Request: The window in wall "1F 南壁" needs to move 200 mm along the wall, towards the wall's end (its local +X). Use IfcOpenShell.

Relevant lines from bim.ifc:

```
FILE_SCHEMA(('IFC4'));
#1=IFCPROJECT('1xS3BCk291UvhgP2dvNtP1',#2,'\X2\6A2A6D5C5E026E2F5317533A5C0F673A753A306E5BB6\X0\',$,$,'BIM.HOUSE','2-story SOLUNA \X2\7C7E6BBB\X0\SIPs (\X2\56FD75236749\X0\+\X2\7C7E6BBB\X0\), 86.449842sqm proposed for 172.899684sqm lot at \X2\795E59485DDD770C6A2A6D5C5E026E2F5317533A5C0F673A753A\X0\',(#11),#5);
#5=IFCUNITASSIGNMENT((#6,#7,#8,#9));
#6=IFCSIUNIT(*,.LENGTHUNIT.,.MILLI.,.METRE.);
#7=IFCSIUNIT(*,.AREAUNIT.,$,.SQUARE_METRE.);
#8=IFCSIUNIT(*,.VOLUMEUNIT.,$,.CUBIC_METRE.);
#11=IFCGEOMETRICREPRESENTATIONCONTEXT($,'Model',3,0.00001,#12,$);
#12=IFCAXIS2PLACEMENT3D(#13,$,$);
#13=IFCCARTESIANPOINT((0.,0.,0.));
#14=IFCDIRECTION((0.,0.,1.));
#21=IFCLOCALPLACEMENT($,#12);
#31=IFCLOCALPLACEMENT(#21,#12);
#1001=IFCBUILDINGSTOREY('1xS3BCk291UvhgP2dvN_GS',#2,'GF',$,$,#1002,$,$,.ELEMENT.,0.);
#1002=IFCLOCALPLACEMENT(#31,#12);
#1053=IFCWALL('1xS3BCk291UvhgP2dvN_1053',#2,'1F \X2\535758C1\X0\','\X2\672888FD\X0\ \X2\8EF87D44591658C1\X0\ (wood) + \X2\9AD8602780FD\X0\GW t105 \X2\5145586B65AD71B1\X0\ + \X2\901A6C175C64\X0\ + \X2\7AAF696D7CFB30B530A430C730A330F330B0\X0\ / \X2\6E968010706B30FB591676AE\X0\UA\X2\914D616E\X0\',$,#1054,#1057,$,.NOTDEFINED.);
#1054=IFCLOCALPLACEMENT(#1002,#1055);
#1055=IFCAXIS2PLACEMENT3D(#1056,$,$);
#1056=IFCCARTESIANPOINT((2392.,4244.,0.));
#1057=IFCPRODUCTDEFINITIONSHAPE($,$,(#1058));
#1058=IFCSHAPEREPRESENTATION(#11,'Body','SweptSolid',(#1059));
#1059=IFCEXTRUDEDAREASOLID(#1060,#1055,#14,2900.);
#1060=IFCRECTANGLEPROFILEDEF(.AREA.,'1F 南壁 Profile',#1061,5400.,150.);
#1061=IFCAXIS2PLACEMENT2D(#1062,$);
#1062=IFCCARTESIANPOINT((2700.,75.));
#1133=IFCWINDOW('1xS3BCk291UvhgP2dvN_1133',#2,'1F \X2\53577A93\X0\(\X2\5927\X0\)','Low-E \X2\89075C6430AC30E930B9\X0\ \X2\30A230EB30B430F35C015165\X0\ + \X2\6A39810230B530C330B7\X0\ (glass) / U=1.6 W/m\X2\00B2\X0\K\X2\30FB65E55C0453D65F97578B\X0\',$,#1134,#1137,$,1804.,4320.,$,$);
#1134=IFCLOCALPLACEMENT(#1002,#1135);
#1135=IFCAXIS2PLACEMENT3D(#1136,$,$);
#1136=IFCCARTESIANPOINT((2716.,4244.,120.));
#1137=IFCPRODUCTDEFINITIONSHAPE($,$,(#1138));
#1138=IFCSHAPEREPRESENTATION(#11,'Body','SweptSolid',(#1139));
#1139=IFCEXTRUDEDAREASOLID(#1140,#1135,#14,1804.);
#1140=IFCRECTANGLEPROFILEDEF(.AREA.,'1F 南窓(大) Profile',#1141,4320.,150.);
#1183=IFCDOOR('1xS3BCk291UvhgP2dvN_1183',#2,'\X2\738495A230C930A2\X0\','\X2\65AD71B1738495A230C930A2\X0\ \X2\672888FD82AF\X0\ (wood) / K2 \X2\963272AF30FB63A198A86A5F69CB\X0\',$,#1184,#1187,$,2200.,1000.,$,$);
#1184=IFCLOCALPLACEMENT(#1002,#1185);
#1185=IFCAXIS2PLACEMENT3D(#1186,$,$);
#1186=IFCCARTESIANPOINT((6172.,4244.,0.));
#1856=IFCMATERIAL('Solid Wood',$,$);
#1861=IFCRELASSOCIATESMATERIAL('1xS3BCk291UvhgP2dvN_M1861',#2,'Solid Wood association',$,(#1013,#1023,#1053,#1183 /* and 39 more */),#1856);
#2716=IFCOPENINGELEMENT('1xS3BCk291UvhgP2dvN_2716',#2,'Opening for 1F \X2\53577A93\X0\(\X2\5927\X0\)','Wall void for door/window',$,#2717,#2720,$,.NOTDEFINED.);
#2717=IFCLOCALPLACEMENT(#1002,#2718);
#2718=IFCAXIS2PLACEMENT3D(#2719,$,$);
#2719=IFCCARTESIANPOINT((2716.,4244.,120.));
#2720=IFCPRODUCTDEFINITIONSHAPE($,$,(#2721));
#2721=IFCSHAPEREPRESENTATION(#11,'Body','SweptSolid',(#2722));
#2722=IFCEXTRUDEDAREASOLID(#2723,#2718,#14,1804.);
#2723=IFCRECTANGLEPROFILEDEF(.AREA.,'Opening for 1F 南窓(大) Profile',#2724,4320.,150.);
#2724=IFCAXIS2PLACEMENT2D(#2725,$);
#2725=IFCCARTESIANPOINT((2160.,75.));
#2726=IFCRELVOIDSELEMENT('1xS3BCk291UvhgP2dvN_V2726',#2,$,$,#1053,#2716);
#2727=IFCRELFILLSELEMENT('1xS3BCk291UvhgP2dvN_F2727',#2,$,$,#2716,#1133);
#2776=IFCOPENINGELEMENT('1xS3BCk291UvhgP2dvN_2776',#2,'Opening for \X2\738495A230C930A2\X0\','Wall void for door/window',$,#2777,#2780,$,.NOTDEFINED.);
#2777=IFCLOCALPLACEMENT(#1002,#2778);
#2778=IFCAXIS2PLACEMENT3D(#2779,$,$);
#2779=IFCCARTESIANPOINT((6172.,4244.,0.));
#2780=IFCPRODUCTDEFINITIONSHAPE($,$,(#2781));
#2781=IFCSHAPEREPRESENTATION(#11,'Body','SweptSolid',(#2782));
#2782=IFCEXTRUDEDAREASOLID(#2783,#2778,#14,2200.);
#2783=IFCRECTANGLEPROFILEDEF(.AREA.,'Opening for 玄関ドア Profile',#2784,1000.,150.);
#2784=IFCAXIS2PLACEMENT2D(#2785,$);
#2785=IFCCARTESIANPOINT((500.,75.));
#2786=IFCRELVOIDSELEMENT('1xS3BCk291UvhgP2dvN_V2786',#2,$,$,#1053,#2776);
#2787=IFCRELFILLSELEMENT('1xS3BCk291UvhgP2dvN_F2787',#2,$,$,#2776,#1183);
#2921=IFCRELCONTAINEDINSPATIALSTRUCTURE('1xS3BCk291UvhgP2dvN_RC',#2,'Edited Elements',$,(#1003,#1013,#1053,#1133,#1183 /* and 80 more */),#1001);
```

```python
import ifcopenshell
import ifcopenshell.api.geometry
import ifcopenshell.util.placement
import ifcopenshell.util.unit

model = ifcopenshell.open("bim.ifc")
unit_scale = ifcopenshell.util.unit.calculate_unit_scale(model)

window = model.by_guid("1xS3BCk291UvhgP2dvN_1133")
opening = window.FillsVoids[0].RelatingOpeningElement
wall = opening.VoidsElements[0].RelatingBuildingElement

wall_matrix = ifcopenshell.util.placement.get_local_placement(wall.ObjectPlacement)
shift = wall_matrix[:3, 0] * 0.2 / unit_scale
before = ifcopenshell.util.placement.get_local_placement(window.ObjectPlacement)[:3, 3].copy()

# The window is not placed relative to its opening, so move both.
for product in (opening, window):
    matrix = ifcopenshell.util.placement.get_local_placement(product.ObjectPlacement)
    matrix[:3, 3] += shift
    ifcopenshell.api.geometry.edit_object_placement(model, product=product, matrix=matrix, is_si=False)

after = ifcopenshell.util.placement.get_local_placement(window.ObjectPlacement)[:3, 3]
print("window moved by", (after - before).round(3) + 0.0)

model.write("bim_updated.ifc")
```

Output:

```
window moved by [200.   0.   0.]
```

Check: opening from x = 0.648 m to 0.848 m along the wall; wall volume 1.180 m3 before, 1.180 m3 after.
